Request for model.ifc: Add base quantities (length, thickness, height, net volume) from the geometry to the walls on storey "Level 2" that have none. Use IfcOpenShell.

First a look at what the model holds.

```python
import ifcopenshell
import ifcopenshell.util.element
import ifcopenshell.util.unit

model = ifcopenshell.open("model.ifc")
print(model.schema)
for unit_type in ("LENGTHUNIT", "AREAUNIT", "VOLUMEUNIT"):
    print(unit_type, ifcopenshell.util.unit.calculate_unit_scale(model, unit_type))
storey = next(s for s in model.by_type("IfcBuildingStorey") if s.Name == "Level 2")
walls = [e for e in ifcopenshell.util.element.get_decomposition(storey) if e.is_a("IfcWall")]
for e in sorted(walls, key=lambda e: e.id()):
    print(e.id(), e.is_a(), e.Name, list(ifcopenshell.util.element.get_psets(e, qtos_only=True)), sep=" | ")
```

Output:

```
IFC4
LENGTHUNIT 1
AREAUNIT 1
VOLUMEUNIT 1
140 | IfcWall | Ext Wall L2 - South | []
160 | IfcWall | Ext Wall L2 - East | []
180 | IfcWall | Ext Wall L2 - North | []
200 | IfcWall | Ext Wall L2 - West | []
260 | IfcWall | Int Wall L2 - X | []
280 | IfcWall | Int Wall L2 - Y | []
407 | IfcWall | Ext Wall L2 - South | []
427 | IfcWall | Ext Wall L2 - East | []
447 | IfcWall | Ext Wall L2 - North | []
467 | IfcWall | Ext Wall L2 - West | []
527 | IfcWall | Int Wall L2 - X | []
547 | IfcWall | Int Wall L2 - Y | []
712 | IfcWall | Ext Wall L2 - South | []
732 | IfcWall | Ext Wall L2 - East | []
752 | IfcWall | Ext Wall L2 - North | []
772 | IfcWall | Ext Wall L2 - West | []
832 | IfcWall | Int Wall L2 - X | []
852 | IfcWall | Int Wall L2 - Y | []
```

```python
import ifcopenshell
import ifcopenshell.api.pset
import ifcopenshell.geom
import ifcopenshell.util.element
import ifcopenshell.util.shape
import ifcopenshell.util.unit

model = ifcopenshell.open("model.ifc")
unit_scale = ifcopenshell.util.unit.calculate_unit_scale(model)
volume_scale = ifcopenshell.util.unit.calculate_unit_scale(model, "VOLUMEUNIT")
settings = ifcopenshell.geom.settings()

storey = next(s for s in model.by_type("IfcBuildingStorey") if s.Name == "Level 2")
walls = [e for e in ifcopenshell.util.element.get_decomposition(storey) if e.is_a("IfcWall")]

for e in sorted(walls, key=lambda e: e.id()):
    if ifcopenshell.util.element.get_psets(e, qtos_only=True, should_inherit=False):
        continue
    # Geometry comes back in metres, in the element's own axes.
    shape = ifcopenshell.geom.create_shape(settings, e)
    values = {
        "Length": ifcopenshell.util.shape.get_x(shape.geometry) / unit_scale,
        "Width": ifcopenshell.util.shape.get_y(shape.geometry) / unit_scale,
        "Height": ifcopenshell.util.shape.get_z(shape.geometry) / unit_scale,
        "NetVolume": ifcopenshell.util.shape.get_volume(shape.geometry) / volume_scale,
    }
    qto = ifcopenshell.api.pset.add_qto(model, product=e, name="Qto_WallBaseQuantities")
    ifcopenshell.api.pset.edit_qto(model, qto=qto, properties=values)
    print(e.id(), {k: round(v, 3) for k, v in values.items()})

model.write("model_v2.ifc")
```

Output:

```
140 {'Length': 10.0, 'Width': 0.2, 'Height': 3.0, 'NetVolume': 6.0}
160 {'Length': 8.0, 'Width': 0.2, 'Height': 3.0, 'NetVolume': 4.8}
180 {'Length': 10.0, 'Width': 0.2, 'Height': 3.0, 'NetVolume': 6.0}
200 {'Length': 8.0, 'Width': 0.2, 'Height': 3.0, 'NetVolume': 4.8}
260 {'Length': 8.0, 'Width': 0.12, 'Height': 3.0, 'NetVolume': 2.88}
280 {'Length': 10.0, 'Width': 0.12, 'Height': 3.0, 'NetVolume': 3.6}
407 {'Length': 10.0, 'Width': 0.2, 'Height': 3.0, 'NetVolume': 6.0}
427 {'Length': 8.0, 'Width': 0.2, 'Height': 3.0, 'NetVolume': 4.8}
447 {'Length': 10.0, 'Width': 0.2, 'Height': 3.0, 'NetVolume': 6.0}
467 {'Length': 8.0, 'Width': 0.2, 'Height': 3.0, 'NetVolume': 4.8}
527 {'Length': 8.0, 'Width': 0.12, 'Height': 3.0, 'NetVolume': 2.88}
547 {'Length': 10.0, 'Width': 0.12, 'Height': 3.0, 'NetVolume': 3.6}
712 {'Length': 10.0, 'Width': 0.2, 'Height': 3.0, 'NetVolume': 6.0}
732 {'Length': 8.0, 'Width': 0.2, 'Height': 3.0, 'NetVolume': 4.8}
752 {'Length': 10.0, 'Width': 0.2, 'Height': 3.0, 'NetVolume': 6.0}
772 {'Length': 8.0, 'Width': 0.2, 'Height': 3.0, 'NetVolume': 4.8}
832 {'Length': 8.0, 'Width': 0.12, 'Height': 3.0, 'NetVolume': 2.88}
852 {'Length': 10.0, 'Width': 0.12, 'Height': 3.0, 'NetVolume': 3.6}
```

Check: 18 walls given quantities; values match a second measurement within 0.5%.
